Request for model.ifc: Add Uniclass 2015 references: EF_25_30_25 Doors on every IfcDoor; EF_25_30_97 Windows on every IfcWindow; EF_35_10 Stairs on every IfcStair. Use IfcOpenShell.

First a look at what the model holds.

```python
import ifcopenshell

model = ifcopenshell.open("model.ifc")
print(model.schema)
print("classifications:", [c.Name for c in model.by_type("IfcClassification")])
for ifc_class in ("IfcDoor", "IfcRoof", "IfcStair", "IfcWall", "IfcWindow"):
    print(ifc_class, len(model.by_type(ifc_class)))
```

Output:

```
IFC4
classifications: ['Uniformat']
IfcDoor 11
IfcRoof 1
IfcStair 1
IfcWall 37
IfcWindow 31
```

```python
import ifcopenshell
import ifcopenshell.api.classification

model = ifcopenshell.open("model.ifc")

system = ifcopenshell.api.classification.add_classification(model, classification="Uniclass 2015")

codes = {
    "IfcDoor": ("EF_25_30_25", "Doors"),
    "IfcWindow": ("EF_25_30_97", "Windows"),
    "IfcStair": ("EF_35_10", "Stairs"),
}
for ifc_class, (code, name) in codes.items():
    products = model.by_type(ifc_class)
    ifcopenshell.api.classification.add_reference(
        model, products=products, classification=system, identification=code, name=name
    )
    print(code, len(products))

model.write("model_updated.ifc")
```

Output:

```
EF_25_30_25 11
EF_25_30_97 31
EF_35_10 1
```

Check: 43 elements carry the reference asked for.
